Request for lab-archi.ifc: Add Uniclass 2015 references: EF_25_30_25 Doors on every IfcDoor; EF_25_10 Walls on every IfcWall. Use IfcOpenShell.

First a look at what the model holds.

```python
import ifcopenshell

model = ifcopenshell.open("lab-archi.ifc")
print(model.schema)
print("classifications:", [c.Name for c in model.by_type("IfcClassification")])
for ifc_class in ("IfcDoor", "IfcRoof", "IfcStair", "IfcWall", "IfcWindow"):
    print(ifc_class, len(model.by_type(ifc_class)))
```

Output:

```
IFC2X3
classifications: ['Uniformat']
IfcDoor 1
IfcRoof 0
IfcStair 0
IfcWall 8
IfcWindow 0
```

```python
import ifcopenshell
import ifcopenshell.api.classification

model = ifcopenshell.open("lab-archi.ifc")

# IFC2X3 requires Source and Edition and has no link from the project to the system.
system = model.create_entity("IfcClassification", Source="NBS", Edition="2015", Name="Uniclass 2015")

codes = {
    "IfcDoor": ("EF_25_30_25", "Doors"),
    "IfcWall": ("EF_25_10", "Walls"),
}
for ifc_class, (code, name) in codes.items():
    products = model.by_type(ifc_class)
    ifcopenshell.api.classification.add_reference(
        model, products=products, classification=system, identification=code, name=name
    )
    print(code, len(products))

model.write("lab-archi_updated.ifc")
```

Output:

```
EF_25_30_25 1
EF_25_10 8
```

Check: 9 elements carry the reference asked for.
